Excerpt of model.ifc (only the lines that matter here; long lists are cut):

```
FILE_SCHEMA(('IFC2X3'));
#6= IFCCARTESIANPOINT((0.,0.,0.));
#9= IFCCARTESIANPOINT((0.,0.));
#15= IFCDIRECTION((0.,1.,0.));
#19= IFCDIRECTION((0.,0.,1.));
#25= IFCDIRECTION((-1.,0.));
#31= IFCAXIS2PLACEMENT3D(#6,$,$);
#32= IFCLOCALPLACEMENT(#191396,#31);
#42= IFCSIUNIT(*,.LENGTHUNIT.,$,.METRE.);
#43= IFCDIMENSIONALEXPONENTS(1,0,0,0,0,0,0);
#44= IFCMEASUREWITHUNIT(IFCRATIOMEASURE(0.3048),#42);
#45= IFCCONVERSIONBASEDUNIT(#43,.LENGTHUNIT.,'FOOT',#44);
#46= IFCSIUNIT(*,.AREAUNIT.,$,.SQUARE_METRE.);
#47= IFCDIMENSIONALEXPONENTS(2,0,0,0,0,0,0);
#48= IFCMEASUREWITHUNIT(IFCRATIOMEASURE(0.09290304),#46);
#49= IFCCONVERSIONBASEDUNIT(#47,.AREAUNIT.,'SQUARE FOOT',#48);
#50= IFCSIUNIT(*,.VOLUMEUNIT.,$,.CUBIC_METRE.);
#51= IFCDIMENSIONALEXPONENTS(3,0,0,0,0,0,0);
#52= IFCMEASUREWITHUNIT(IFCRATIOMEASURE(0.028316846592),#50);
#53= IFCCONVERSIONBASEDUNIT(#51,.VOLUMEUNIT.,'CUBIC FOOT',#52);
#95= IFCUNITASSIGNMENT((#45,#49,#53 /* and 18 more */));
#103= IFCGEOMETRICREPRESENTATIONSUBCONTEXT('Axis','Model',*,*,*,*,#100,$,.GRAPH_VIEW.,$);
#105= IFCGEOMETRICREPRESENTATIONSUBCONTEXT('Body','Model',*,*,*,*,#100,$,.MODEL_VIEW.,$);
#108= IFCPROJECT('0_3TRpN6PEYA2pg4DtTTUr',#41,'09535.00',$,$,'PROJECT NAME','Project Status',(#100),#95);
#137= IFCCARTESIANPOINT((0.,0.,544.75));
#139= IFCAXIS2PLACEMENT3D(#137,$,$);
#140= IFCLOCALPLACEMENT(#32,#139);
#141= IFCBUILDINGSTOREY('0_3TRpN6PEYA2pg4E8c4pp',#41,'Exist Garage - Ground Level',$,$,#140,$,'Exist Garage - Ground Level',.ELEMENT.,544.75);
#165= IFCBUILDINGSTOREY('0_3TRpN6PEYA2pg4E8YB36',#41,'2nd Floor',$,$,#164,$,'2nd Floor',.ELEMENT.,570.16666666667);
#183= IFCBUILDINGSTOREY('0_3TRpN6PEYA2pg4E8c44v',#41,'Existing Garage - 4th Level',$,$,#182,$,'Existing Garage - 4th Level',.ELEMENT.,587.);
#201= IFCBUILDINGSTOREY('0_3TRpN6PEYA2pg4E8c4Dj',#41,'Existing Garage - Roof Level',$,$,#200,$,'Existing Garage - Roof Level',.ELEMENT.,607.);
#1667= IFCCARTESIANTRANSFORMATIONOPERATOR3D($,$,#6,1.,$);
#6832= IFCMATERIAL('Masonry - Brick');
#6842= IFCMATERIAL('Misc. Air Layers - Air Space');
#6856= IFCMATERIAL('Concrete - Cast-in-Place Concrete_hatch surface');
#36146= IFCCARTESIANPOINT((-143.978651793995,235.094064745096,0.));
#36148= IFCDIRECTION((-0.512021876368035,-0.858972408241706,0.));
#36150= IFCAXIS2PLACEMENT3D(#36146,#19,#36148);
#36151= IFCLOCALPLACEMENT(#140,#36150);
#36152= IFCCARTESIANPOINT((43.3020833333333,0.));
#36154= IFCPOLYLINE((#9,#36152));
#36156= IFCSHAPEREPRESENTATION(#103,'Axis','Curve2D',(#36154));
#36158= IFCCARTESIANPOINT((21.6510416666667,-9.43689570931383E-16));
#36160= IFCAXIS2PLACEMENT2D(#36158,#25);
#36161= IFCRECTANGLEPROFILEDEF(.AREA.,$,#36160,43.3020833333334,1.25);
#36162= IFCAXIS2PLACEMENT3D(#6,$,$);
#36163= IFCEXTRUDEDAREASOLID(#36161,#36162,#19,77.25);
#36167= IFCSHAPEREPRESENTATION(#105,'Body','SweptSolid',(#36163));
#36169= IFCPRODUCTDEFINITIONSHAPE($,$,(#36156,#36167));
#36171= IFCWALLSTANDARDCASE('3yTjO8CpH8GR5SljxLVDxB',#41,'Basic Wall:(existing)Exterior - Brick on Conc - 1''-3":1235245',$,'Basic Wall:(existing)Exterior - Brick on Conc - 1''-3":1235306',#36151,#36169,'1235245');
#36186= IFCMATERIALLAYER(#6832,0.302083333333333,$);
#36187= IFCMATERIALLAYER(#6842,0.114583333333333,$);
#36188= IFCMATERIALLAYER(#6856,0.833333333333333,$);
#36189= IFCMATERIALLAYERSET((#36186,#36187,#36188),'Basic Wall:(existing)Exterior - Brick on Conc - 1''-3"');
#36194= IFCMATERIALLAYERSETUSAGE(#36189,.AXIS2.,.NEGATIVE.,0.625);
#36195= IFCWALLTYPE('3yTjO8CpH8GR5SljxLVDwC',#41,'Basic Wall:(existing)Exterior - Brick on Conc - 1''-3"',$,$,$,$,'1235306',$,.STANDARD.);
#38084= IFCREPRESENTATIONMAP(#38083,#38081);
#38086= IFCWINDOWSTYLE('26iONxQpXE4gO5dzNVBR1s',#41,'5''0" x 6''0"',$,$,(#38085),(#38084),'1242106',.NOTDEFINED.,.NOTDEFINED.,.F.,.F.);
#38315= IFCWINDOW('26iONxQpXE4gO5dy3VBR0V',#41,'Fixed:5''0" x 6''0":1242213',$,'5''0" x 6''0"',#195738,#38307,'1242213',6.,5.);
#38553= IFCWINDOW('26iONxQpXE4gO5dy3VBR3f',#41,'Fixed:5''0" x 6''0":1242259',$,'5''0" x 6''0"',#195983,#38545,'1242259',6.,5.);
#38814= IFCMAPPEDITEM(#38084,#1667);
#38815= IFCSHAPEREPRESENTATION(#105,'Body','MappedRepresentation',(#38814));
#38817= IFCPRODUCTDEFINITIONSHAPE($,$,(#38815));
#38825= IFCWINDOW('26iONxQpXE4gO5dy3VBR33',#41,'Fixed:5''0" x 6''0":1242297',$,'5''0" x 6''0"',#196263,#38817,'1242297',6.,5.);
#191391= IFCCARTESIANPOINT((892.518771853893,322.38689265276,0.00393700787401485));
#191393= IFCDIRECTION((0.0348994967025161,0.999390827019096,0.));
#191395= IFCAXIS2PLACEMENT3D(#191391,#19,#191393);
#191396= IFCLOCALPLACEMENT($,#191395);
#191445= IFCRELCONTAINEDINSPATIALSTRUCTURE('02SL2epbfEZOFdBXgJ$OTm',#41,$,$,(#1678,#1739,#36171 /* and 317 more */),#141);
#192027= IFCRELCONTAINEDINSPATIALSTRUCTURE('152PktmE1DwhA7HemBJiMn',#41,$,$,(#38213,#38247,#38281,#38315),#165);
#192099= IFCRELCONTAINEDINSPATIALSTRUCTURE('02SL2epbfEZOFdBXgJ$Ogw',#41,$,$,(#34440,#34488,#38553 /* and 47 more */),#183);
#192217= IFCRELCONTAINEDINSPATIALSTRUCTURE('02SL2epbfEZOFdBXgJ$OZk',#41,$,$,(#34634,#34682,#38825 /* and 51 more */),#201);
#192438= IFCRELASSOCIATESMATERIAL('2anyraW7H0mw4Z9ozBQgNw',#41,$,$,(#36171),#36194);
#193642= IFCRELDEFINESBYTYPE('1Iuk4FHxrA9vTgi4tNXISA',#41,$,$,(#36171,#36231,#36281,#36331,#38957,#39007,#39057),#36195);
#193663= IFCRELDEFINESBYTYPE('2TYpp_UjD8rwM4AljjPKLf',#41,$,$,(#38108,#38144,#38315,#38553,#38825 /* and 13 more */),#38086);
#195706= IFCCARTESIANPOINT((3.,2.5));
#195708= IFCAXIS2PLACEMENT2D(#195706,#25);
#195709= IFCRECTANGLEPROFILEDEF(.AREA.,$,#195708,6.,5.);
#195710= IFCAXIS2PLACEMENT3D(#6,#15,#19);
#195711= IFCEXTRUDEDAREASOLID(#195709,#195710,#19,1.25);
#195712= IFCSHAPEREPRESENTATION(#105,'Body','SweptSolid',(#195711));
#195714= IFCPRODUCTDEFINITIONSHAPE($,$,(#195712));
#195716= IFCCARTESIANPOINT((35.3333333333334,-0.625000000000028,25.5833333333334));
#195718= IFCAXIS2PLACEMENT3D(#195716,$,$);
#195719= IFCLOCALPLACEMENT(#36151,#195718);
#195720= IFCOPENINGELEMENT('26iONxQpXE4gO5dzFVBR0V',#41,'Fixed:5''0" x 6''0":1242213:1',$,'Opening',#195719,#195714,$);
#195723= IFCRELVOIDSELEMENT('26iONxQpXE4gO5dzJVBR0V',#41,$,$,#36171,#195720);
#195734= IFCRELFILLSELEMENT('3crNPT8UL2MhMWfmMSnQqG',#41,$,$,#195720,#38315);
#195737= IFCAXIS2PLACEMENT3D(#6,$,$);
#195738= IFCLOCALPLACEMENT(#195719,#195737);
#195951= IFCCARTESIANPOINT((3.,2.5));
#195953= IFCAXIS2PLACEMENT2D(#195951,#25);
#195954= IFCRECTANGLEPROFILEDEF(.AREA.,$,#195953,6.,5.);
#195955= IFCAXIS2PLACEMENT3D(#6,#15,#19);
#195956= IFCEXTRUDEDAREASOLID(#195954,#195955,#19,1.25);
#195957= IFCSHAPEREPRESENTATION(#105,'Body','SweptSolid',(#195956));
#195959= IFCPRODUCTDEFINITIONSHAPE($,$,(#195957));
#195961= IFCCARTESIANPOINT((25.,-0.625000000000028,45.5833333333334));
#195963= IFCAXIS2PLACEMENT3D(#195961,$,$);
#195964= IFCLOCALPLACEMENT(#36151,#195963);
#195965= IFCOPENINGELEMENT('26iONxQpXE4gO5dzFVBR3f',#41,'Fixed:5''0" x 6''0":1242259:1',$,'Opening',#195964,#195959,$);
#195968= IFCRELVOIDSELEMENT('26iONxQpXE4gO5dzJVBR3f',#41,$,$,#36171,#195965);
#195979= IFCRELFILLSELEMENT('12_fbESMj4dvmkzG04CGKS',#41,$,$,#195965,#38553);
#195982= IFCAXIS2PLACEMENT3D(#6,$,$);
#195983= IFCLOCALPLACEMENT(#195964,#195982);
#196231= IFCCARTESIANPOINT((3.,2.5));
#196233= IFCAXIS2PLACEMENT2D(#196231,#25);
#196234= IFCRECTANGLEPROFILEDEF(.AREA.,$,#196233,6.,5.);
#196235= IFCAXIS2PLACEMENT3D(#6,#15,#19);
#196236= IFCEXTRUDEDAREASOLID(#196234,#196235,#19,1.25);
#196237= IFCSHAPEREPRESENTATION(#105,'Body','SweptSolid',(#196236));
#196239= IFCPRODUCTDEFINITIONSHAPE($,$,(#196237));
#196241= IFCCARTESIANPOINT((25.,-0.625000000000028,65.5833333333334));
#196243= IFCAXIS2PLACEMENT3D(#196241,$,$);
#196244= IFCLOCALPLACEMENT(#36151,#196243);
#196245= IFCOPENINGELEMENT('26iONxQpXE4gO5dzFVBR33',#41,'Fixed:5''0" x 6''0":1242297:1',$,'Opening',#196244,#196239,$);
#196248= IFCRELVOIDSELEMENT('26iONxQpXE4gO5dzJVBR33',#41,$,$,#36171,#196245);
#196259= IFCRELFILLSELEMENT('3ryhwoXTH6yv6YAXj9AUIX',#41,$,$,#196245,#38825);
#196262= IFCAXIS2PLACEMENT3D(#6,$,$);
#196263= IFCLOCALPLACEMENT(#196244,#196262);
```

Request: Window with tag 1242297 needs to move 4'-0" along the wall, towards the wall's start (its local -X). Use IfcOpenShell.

```python
import ifcopenshell
import ifcopenshell.api.geometry
import ifcopenshell.util.placement
import ifcopenshell.util.unit

model = ifcopenshell.open("model.ifc")
unit_scale = ifcopenshell.util.unit.calculate_unit_scale(model)

window = model.by_guid("26iONxQpXE4gO5dy3VBR33")
opening = window.FillsVoids[0].RelatingOpeningElement
wall = opening.VoidsElements[0].RelatingBuildingElement

wall_matrix = ifcopenshell.util.placement.get_local_placement(wall.ObjectPlacement)
shift = wall_matrix[:3, 0] * -48 * 0.0254 / unit_scale
before = ifcopenshell.util.placement.get_local_placement(window.ObjectPlacement)[:3, 3].copy()

# The window is placed relative to its opening, so it follows when the opening moves.
matrix = ifcopenshell.util.placement.get_local_placement(opening.ObjectPlacement)
matrix[:3, 3] += shift
ifcopenshell.api.geometry.edit_object_placement(
    model, product=opening, matrix=matrix, is_si=False, should_transform_children=True
)

after = ifcopenshell.util.placement.get_local_placement(window.ObjectPlacement)[:3, 3]
print("window moved by", (after - before).round(3) + 0.0)

model.write("model_updated.ifc")
```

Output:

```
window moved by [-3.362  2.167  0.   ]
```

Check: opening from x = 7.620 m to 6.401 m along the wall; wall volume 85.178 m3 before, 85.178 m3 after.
